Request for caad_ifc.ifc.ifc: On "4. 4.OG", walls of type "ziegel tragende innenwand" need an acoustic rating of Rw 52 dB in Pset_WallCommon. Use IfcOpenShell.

First a look at what the model holds.

```python
import ifcopenshell
import ifcopenshell.util.element

model = ifcopenshell.open("caad_ifc.ifc.ifc")
print(model.schema)
storey = next(s for s in model.by_type("IfcBuildingStorey") if s.Name == "4. 4.OG")
walls = [e for e in ifcopenshell.util.element.get_decomposition(storey) if e.is_a("IfcWall")]
seen = {}
for e in walls:
    element_type = ifcopenshell.util.element.get_type(e)
    key = (element_type.Name if element_type != e and element_type else None, ifcopenshell.util.element.get_pset(e, "Pset_WallCommon", "AcousticRating"))
    seen[key] = seen.get(key, 0) + 1
for (name, value), count in sorted(seen.items(), key=str):
    print(count, "x", name, "|", value)
```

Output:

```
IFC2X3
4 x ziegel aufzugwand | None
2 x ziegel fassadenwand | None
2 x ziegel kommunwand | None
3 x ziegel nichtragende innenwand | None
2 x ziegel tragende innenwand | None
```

```python
import ifcopenshell
import ifcopenshell.api.pset
import ifcopenshell.util.element

model = ifcopenshell.open("caad_ifc.ifc.ifc")

storey = next(s for s in model.by_type("IfcBuildingStorey") if s.Name == "4. 4.OG")
walls = [e for e in ifcopenshell.util.element.get_decomposition(storey) if e.is_a("IfcWall")]

count = 0
for e in walls:
    element_type = ifcopenshell.util.element.get_type(e)
    if element_type in (None, e) or element_type.Name != "ziegel tragende innenwand":
        continue
    # add_pset returns the element's existing set when there is one.
    pset = ifcopenshell.api.pset.add_pset(model, product=e, name="Pset_WallCommon")
    ifcopenshell.api.pset.edit_pset(model, pset=pset, properties={"AcousticRating": "Rw 52 dB"})
    count += 1

print(count, "walls updated")

model.write("caad_ifc.ifc-out.ifc")
```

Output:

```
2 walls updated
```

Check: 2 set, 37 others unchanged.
